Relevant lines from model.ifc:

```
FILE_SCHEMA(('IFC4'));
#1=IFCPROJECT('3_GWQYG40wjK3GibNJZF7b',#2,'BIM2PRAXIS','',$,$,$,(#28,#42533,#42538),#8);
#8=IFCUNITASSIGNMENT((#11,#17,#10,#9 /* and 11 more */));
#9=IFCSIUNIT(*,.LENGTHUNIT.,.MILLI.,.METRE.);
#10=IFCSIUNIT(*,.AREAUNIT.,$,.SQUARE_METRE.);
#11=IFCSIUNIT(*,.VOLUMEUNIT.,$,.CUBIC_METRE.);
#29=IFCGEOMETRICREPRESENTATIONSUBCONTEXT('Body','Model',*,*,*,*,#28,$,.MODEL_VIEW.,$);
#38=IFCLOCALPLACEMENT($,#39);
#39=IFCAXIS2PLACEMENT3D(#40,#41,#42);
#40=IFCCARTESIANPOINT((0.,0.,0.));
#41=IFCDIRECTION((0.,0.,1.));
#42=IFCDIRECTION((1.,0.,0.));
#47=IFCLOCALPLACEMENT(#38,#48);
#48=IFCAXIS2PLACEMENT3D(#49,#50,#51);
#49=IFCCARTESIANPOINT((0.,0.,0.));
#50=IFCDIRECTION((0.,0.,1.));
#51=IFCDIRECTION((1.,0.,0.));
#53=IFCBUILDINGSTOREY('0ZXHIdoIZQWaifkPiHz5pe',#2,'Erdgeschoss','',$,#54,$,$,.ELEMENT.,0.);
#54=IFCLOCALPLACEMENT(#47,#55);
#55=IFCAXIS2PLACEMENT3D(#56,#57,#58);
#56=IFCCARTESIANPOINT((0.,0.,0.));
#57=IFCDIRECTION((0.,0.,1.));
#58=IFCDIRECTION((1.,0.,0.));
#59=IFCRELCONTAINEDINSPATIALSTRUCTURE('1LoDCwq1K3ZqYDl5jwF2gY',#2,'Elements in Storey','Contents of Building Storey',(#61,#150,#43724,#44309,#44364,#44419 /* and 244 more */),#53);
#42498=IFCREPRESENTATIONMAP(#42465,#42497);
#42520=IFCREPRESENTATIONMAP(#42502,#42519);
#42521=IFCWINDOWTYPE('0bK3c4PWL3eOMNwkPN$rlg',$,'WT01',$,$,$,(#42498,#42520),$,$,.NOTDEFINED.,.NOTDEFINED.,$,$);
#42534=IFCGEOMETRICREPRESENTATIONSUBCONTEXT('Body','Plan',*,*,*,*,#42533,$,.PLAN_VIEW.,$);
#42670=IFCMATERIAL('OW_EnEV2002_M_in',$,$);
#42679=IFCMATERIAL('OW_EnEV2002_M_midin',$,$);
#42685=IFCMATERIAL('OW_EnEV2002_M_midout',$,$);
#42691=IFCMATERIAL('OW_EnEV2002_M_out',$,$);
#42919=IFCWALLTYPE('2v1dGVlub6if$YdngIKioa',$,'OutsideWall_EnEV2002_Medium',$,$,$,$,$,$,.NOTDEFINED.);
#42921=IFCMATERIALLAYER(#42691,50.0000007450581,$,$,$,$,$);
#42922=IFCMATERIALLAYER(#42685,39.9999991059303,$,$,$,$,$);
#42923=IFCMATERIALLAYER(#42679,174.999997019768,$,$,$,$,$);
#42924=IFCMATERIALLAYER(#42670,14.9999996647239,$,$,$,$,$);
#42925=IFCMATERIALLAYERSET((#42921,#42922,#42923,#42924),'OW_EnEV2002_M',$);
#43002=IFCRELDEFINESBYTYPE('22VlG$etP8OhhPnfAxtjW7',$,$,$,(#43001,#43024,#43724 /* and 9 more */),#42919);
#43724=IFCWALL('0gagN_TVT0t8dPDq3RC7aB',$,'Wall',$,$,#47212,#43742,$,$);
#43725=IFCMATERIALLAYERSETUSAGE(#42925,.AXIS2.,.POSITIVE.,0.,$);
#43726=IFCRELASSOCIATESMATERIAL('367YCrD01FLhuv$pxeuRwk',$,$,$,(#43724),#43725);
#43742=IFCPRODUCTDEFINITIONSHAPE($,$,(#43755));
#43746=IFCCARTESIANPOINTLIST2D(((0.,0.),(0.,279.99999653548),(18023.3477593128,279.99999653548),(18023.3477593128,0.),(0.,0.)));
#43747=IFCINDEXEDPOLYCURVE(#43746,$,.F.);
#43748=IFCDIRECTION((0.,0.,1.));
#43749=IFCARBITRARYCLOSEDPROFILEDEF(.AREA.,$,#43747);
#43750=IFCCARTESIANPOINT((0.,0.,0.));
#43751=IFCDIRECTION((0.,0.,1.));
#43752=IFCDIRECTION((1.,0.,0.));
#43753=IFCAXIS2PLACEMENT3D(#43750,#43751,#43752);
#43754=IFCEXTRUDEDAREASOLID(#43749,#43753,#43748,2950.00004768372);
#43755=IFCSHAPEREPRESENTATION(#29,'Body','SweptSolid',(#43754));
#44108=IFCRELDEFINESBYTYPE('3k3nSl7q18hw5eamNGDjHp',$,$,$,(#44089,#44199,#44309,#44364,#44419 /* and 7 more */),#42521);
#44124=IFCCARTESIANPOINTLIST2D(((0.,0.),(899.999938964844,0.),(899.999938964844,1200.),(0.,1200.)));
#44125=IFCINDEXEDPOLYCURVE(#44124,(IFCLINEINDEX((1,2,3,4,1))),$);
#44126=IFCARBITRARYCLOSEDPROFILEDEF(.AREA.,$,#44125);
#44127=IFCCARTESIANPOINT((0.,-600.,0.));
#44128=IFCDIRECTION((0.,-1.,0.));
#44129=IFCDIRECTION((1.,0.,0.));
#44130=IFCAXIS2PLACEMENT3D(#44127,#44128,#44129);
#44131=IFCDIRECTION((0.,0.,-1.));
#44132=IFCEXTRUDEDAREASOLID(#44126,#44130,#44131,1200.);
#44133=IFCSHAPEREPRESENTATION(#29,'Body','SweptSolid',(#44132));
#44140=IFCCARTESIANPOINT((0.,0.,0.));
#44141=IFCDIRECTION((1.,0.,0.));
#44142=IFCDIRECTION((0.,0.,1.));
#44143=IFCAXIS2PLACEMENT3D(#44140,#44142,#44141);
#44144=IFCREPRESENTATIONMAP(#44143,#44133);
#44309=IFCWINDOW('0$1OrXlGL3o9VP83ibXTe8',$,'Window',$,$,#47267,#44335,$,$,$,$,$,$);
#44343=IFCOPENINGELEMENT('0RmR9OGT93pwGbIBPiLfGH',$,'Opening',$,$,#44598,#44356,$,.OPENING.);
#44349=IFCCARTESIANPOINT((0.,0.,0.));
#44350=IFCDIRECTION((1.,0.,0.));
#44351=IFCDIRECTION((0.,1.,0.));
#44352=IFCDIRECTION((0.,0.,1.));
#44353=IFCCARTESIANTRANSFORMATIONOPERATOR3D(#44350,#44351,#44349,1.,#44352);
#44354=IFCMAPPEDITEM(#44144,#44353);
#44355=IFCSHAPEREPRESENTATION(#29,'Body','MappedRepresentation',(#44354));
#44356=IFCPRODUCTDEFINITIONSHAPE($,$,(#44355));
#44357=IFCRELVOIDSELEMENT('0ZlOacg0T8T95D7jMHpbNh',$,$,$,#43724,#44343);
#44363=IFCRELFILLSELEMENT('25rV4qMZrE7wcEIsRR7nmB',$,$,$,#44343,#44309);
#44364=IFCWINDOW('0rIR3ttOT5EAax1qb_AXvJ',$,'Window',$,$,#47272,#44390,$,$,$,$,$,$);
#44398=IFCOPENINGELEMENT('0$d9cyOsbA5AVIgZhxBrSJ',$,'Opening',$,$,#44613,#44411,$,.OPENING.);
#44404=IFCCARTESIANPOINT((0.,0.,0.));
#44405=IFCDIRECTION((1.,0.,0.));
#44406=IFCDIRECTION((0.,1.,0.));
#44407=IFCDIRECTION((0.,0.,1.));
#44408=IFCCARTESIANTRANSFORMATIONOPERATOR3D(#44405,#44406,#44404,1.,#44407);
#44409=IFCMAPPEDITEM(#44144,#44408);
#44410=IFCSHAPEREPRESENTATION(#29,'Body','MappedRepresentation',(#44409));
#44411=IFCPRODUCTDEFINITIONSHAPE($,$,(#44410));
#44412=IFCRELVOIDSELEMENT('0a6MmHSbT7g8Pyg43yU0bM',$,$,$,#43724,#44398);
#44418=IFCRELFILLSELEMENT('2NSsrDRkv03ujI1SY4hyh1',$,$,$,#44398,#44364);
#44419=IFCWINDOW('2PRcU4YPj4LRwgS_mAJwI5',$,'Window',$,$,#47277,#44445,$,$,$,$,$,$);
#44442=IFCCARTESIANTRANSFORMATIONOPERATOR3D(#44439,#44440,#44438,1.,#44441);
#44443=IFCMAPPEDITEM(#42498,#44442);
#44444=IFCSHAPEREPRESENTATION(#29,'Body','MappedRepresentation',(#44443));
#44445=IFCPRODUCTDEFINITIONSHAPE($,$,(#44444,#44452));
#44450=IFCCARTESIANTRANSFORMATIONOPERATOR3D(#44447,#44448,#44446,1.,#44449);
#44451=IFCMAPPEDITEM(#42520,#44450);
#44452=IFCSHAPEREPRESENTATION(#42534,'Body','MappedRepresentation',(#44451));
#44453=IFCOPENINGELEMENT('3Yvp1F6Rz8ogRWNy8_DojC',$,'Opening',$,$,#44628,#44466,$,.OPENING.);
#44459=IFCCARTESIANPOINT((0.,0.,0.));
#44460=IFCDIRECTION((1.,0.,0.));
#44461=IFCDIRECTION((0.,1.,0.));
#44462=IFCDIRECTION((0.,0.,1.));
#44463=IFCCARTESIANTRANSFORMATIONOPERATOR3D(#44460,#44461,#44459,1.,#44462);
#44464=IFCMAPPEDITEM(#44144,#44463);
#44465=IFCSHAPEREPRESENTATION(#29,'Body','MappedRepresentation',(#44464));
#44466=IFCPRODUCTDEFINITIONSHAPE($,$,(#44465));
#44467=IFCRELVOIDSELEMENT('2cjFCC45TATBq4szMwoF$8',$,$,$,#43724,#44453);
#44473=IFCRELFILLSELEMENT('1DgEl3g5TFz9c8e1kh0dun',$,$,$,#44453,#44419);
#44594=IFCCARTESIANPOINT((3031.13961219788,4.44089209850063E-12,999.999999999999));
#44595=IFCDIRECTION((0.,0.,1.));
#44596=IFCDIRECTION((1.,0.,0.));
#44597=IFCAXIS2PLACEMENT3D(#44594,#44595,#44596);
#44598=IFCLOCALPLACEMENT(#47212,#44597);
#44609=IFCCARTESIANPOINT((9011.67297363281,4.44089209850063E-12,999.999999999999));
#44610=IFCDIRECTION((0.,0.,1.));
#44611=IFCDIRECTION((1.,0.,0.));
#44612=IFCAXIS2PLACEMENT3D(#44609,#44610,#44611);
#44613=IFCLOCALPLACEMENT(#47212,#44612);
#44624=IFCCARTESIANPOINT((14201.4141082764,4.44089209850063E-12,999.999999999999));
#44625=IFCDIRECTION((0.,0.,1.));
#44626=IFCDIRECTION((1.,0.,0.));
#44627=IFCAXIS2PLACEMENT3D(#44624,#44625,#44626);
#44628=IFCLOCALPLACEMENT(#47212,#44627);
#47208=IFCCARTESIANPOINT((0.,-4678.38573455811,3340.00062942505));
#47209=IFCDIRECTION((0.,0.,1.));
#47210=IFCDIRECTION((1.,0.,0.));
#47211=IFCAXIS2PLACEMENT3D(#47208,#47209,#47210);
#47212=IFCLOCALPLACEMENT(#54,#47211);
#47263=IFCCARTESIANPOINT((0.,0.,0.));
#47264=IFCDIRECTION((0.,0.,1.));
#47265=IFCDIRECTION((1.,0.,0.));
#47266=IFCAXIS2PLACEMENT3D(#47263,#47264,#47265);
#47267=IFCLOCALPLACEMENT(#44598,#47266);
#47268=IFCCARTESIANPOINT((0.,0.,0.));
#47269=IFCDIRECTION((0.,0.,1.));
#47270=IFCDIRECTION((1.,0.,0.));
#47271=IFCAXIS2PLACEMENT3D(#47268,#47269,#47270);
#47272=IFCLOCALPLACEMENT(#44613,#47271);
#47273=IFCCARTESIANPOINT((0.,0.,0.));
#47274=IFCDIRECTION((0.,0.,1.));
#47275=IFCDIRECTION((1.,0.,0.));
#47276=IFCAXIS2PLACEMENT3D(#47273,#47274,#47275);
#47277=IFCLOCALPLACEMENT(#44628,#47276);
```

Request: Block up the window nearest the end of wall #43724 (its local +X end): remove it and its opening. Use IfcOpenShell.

```python
import ifcopenshell
import ifcopenshell.api.feature
import ifcopenshell.api.root
import ifcopenshell.geom
import ifcopenshell.util.shape

model = ifcopenshell.open("model.ifc")
settings = ifcopenshell.geom.settings()


def volume(element):
    """Net volume in cubic metres, openings subtracted."""
    shape = ifcopenshell.geom.create_shape(settings, element)
    return ifcopenshell.util.shape.get_volume(shape.geometry)


window = model.by_guid("2PRcU4YPj4LRwgS_mAJwI5")
opening = window.FillsVoids[0].RelatingOpeningElement
wall = opening.VoidsElements[0].RelatingBuildingElement
before = volume(wall)

ifcopenshell.api.root.remove_product(model, product=window)
ifcopenshell.api.feature.remove_feature(model, feature=opening)

after = volume(wall)

print(f"wall volume {before:.3f} -> {after:.3f} m3")

model.write("model_v2.ifc")
```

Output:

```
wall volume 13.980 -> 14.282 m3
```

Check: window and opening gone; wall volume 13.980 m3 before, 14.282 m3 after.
